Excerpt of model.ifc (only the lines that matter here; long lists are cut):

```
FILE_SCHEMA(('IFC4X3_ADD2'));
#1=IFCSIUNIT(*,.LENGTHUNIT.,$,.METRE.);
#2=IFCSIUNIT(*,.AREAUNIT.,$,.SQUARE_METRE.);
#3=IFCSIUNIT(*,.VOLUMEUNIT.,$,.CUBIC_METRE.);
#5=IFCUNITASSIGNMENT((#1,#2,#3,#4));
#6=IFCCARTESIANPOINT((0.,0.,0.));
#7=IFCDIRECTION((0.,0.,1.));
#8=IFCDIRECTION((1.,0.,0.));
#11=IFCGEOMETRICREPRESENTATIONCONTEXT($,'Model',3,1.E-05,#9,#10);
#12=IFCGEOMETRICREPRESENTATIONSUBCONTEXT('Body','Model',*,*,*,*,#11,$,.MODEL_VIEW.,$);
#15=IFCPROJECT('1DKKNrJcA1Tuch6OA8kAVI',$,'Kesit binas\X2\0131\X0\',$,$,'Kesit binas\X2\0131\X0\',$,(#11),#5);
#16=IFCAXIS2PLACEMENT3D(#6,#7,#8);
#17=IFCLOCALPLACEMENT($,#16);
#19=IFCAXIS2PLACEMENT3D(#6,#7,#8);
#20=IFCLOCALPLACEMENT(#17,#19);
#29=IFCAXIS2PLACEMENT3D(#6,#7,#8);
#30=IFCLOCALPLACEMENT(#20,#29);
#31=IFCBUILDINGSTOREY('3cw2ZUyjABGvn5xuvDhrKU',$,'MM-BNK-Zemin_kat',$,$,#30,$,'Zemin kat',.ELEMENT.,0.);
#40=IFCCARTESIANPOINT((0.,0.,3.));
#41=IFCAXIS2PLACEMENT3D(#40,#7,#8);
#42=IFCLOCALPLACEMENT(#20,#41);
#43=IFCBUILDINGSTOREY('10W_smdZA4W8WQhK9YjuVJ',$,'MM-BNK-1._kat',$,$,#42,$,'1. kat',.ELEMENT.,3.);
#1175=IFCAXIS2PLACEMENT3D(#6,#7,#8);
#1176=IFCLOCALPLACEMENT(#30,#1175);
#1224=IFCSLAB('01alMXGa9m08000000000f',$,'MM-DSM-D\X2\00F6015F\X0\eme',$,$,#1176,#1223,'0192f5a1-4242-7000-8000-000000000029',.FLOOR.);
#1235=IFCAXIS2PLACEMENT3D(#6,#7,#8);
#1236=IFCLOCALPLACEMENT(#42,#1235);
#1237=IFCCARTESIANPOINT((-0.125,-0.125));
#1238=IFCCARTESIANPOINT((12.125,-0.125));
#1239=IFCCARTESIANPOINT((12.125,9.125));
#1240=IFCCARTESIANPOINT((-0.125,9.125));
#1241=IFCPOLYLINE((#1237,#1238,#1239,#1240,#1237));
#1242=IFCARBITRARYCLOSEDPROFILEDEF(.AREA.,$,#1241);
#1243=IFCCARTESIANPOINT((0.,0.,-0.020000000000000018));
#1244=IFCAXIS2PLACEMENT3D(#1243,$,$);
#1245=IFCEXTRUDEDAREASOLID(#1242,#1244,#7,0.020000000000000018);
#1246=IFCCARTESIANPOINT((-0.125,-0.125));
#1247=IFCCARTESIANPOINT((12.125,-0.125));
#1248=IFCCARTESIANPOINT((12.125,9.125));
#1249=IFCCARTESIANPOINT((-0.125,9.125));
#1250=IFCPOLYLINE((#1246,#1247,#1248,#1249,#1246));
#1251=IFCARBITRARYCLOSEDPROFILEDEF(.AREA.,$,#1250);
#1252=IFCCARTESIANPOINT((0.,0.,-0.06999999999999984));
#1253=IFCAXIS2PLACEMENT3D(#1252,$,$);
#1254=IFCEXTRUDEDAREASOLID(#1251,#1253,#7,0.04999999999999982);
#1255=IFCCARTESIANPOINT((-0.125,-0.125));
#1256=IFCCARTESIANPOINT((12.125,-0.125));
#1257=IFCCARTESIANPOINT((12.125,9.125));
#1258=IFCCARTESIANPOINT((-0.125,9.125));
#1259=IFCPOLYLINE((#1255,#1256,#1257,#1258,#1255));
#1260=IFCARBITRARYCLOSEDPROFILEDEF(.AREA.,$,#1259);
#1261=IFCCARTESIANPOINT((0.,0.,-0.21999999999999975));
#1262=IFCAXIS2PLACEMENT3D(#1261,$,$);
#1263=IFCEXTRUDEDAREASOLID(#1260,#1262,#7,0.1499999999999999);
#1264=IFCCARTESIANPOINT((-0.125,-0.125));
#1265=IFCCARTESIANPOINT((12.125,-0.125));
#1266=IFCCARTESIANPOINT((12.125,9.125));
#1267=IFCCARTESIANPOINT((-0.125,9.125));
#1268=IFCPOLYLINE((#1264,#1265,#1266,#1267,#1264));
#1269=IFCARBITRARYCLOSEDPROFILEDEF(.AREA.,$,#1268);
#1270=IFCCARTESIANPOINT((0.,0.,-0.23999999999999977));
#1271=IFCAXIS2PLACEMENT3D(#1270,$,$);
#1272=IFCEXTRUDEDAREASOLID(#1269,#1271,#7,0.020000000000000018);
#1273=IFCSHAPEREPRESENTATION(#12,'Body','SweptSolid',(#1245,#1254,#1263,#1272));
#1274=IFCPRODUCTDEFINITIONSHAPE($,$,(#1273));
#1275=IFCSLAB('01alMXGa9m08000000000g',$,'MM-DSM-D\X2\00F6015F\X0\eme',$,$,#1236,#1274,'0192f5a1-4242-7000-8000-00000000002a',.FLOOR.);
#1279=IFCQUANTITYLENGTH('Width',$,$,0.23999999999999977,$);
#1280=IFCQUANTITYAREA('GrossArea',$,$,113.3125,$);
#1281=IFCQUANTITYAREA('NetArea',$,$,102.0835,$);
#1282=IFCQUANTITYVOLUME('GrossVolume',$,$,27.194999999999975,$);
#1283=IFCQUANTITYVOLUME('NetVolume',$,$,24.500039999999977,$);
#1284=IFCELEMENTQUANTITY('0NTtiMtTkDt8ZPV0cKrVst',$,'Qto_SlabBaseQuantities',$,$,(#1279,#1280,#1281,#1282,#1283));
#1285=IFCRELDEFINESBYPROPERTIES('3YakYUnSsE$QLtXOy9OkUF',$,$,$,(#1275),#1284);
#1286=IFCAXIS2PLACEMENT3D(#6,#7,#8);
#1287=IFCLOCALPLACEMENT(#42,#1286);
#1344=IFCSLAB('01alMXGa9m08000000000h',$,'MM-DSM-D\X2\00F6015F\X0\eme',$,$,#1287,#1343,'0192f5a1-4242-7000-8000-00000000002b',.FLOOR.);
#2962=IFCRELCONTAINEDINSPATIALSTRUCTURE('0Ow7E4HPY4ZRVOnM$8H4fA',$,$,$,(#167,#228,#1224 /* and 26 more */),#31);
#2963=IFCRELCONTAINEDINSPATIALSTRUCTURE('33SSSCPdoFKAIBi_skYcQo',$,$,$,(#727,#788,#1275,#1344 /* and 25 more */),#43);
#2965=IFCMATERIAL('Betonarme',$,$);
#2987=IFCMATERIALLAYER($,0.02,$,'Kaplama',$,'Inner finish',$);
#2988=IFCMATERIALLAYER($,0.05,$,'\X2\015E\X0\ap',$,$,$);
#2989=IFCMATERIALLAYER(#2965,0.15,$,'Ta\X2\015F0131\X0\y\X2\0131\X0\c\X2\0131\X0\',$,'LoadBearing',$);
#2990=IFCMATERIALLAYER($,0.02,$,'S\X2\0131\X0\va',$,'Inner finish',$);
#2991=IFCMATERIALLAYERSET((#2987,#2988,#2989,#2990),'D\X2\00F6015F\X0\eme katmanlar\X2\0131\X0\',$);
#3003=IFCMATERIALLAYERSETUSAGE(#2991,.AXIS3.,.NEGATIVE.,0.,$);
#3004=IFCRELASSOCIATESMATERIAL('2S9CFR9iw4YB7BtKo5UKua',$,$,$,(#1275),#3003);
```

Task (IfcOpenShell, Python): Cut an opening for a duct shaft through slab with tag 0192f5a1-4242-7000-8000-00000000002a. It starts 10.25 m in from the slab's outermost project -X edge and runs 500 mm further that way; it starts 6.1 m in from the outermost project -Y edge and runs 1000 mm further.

```python
import numpy as np
import ifcopenshell
import ifcopenshell.api.feature
import ifcopenshell.api.geometry
import ifcopenshell.api.pset
import ifcopenshell.api.root
import ifcopenshell.geom
import ifcopenshell.util.element
import ifcopenshell.util.placement
import ifcopenshell.util.representation
import ifcopenshell.util.shape
import ifcopenshell.util.unit

model = ifcopenshell.open("model.ifc")
unit_scale = ifcopenshell.util.unit.calculate_unit_scale(model)
area_scale = ifcopenshell.util.unit.calculate_unit_scale(model, "AREAUNIT")
volume_scale = ifcopenshell.util.unit.calculate_unit_scale(model, "VOLUMEUNIT")
settings = ifcopenshell.geom.settings()


def volume(element):
    """Net volume in cubic metres, openings subtracted."""
    shape = ifcopenshell.geom.create_shape(settings, element)
    return ifcopenshell.util.shape.get_volume(shape.geometry)


slab = model.by_guid("01alMXGa9m08000000000g")
before = volume(slab)

# Extent in the slab's own axes, in metres. The edges named are its -X and -Y sides.
slab_shape = ifcopenshell.geom.create_shape(settings, slab)
vertices = ifcopenshell.util.shape.get_vertices(slab_shape.geometry)
x_min, y_min, bottom = vertices.min(axis=0)
top = vertices[:, 2].max()

opening = ifcopenshell.api.root.create_entity(model, ifc_class="IfcOpeningElement", name="Duct shaft opening", predefined_type="OPENING")
context = ifcopenshell.util.representation.get_context(model, "Model", "Body", "MODEL_VIEW")
width, depth = 0.5, 1
outline = [(0.0, 0.0), (width, 0.0), (width, depth), (0.0, depth), (0.0, 0.0)]
# Overshoot both faces by 50 mm so the cut is clean.
shape = ifcopenshell.api.geometry.add_slab_representation(
    model, context=context, depth=top - bottom + 0.1, polyline=outline
)
ifcopenshell.api.geometry.assign_representation(model, product=opening, representation=shape)

matrix = ifcopenshell.util.placement.get_local_placement(slab.ObjectPlacement)
matrix[:, 3] = matrix @ np.append(np.array([x_min + 10.25, y_min + 6.1, bottom - 0.05]) / unit_scale, 1.0)
ifcopenshell.api.geometry.edit_object_placement(model, product=opening, matrix=matrix, is_si=False)
ifcopenshell.api.feature.add_feature(model, feature=opening, element=slab)

after = volume(slab)

# Update the slab's stored quantities.
qto = model.by_id(ifcopenshell.util.element.get_pset(slab, "Qto_SlabBaseQuantities", should_inherit=False)["id"])
ifcopenshell.api.pset.edit_qto(model, qto=qto, properties={
    "NetArea": after / (top - bottom) / area_scale,
    "NetVolume": after / volume_scale,
})

print(f"slab volume {before:.3f} -> {after:.3f} m3")

model.write("model_rev.ifc")
```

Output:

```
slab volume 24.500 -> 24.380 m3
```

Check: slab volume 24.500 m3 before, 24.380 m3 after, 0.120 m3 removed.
